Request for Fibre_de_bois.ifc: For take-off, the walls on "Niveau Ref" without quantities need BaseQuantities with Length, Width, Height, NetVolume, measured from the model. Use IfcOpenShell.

First a look at what the model holds.

```python
import ifcopenshell
import ifcopenshell.util.element
import ifcopenshell.util.unit

model = ifcopenshell.open("Fibre_de_bois.ifc")
print(model.schema)
for unit_type in ("LENGTHUNIT", "AREAUNIT", "VOLUMEUNIT"):
    print(unit_type, ifcopenshell.util.unit.calculate_unit_scale(model, unit_type))
storey = next(s for s in model.by_type("IfcBuildingStorey") if s.Name == "Niveau Ref")
walls = [e for e in ifcopenshell.util.element.get_decomposition(storey) if e.is_a("IfcWall")]
for e in sorted(walls, key=lambda e: e.id()):
    print(e.id(), e.is_a(), e.Name, list(ifcopenshell.util.element.get_psets(e, qtos_only=True)), sep=" | ")
```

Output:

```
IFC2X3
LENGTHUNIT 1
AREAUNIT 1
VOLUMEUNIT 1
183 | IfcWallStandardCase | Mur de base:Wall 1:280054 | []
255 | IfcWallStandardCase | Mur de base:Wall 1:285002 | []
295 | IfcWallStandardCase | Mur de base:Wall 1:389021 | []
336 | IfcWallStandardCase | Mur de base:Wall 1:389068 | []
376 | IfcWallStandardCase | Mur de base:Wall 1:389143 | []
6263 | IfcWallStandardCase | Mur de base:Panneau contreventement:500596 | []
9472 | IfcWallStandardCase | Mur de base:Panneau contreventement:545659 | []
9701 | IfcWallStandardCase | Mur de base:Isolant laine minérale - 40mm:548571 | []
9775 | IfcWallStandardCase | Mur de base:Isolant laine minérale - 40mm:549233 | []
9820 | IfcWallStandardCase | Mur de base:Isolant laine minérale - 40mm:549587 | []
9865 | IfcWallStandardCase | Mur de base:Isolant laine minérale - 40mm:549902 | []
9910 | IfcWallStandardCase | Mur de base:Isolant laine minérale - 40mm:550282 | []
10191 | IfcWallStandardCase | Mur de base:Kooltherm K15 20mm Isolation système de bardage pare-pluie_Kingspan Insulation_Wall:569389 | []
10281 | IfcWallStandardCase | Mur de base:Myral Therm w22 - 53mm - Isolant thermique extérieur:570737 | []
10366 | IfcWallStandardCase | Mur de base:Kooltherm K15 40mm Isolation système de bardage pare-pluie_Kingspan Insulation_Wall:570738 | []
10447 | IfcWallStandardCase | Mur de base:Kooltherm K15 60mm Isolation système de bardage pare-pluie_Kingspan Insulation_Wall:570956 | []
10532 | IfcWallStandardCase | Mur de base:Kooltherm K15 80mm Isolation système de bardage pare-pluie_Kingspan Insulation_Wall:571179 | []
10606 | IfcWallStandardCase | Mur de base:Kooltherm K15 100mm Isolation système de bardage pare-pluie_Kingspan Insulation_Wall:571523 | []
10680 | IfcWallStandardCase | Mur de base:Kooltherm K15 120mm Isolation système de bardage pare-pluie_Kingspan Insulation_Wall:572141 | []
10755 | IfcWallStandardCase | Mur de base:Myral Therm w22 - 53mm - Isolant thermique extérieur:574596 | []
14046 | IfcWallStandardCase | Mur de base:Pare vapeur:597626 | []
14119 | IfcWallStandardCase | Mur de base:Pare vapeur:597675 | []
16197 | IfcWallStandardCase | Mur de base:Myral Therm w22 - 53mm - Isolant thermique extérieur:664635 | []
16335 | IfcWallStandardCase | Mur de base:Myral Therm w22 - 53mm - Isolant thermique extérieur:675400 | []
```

```python
import ifcopenshell
import ifcopenshell.api.pset
import ifcopenshell.geom
import ifcopenshell.util.element
import ifcopenshell.util.shape
import ifcopenshell.util.unit

model = ifcopenshell.open("Fibre_de_bois.ifc")
unit_scale = ifcopenshell.util.unit.calculate_unit_scale(model)
volume_scale = ifcopenshell.util.unit.calculate_unit_scale(model, "VOLUMEUNIT")
settings = ifcopenshell.geom.settings()

storey = next(s for s in model.by_type("IfcBuildingStorey") if s.Name == "Niveau Ref")
walls = [e for e in ifcopenshell.util.element.get_decomposition(storey) if e.is_a("IfcWall")]

for e in sorted(walls, key=lambda e: e.id()):
    if ifcopenshell.util.element.get_psets(e, qtos_only=True, should_inherit=False):
        continue
    # Geometry comes back in metres, in the element's own axes.
    shape = ifcopenshell.geom.create_shape(settings, e)
    values = {
        "Length": ifcopenshell.util.shape.get_x(shape.geometry) / unit_scale,
        "Width": ifcopenshell.util.shape.get_y(shape.geometry) / unit_scale,
        "Height": ifcopenshell.util.shape.get_z(shape.geometry) / unit_scale,
        "NetVolume": ifcopenshell.util.shape.get_volume(shape.geometry) / volume_scale,
    }
    qto = ifcopenshell.api.pset.add_qto(model, product=e, name="BaseQuantities")
    ifcopenshell.api.pset.edit_qto(model, qto=qto, properties=values)
    print(e.id(), {k: round(v, 3) for k, v in values.items()})

model.write("Fibre_de_bois_v2.ifc")
```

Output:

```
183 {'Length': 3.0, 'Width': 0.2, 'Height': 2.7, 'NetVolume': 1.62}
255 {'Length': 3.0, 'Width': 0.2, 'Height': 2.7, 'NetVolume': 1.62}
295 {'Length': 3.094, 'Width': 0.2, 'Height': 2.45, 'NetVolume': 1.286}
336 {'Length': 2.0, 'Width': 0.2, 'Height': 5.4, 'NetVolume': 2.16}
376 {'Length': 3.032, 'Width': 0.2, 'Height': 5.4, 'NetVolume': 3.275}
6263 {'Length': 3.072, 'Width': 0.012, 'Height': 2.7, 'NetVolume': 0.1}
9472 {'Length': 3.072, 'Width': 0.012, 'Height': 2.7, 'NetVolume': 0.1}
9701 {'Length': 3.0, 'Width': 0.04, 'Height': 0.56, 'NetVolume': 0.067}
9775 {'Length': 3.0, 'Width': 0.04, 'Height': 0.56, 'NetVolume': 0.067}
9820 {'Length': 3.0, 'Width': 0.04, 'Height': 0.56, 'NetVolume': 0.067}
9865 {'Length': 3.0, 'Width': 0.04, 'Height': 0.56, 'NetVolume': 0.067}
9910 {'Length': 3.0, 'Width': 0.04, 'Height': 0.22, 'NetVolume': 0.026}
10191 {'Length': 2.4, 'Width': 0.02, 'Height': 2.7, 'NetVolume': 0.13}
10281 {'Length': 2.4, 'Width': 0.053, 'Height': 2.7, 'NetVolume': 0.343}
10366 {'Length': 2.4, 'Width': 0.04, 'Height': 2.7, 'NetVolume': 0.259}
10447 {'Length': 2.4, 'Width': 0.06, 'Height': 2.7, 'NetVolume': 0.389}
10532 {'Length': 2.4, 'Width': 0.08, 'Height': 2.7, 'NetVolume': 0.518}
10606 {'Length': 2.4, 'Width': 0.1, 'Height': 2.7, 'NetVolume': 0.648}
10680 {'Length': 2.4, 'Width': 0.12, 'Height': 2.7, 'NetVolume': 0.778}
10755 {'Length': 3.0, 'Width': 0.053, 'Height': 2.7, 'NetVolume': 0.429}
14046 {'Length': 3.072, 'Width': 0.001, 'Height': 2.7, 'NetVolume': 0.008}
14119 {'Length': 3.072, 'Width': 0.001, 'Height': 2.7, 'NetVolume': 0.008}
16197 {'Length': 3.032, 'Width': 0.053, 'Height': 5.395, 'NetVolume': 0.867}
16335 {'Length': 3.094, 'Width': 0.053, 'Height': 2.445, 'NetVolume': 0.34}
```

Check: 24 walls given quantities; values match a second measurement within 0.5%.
